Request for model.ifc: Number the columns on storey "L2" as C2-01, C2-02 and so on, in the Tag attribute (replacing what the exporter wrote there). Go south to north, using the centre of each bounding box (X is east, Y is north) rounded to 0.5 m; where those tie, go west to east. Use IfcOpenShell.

First a look at what the model holds.

```python
import ifcopenshell
import ifcopenshell.util.element
import ifcopenshell.util.placement

model = ifcopenshell.open("model.ifc")
print(model.schema)
storey = next(s for s in model.by_type("IfcBuildingStorey") if s.Name == "L2")
columns = [e for e in ifcopenshell.util.element.get_decomposition(storey) if e.is_a("IfcColumn")]
for e in sorted(columns, key=lambda e: e.id()):
    origin = ifcopenshell.util.placement.get_local_placement(e.ObjectPlacement)[:3, 3]
    print(e.id(), e.Tag, e.Name, origin.round(2) + 0.0, sep=" | ")
```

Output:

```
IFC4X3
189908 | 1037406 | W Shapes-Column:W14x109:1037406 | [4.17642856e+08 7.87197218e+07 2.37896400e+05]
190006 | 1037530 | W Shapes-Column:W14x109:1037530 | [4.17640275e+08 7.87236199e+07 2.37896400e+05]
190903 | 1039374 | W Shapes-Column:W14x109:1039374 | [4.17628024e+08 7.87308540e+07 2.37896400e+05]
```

```python
import ifcopenshell
import ifcopenshell.geom
import ifcopenshell.util.element
import ifcopenshell.util.shape

model = ifcopenshell.open("model.ifc")
settings = ifcopenshell.geom.settings()
settings.set("use-world-coords", True)


def centre(element):
    shape = ifcopenshell.geom.create_shape(settings, element)
    return ifcopenshell.util.shape.get_bbox_centroid(shape.geometry)


storey = next(s for s in model.by_type("IfcBuildingStorey") if s.Name == "L2")
columns = [e for e in ifcopenshell.util.element.get_decomposition(storey) if e.is_a("IfcColumn")]

# Insertion points can sit at a corner or the storey origin, so sort by the geometry (in metres).
centres = {e: centre(e) for e in columns}
columns.sort(key=lambda e: (round(centres[e][1] / 0.5), centres[e][0]))

for i, e in enumerate(columns, start=1):
    number = f"C2-{i:02d}"
    e.Tag = number
    print(e.id(), number)

model.write("model_rev.ifc")
```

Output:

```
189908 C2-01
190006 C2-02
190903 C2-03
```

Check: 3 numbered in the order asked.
